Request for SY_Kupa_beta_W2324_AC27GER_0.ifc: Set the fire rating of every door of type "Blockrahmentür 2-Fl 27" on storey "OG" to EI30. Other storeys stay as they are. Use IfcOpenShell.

First a look at what the model holds.

```python
import ifcopenshell
import ifcopenshell.util.element

model = ifcopenshell.open("SY_Kupa_beta_W2324_AC27GER_0.ifc")
print(model.schema)
storey = next(s for s in model.by_type("IfcBuildingStorey") if s.Name == "OG")
doors = [e for e in ifcopenshell.util.element.get_decomposition(storey) if e.is_a("IfcDoor")]
seen = {}
for e in doors:
    element_type = ifcopenshell.util.element.get_type(e)
    key = (element_type.Name if element_type != e and element_type else None, ifcopenshell.util.element.get_pset(e, "Pset_DoorCommon", "FireRating"))
    seen[key] = seen.get(key, 0) + 1
for (name, value), count in sorted(seen.items(), key=str):
    print(count, "x", name, "|", value)
```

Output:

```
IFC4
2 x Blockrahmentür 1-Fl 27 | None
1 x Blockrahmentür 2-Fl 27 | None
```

```python
import ifcopenshell
import ifcopenshell.api.pset
import ifcopenshell.util.element

model = ifcopenshell.open("SY_Kupa_beta_W2324_AC27GER_0.ifc")

storey = next(s for s in model.by_type("IfcBuildingStorey") if s.Name == "OG")
doors = [e for e in ifcopenshell.util.element.get_decomposition(storey) if e.is_a("IfcDoor")]

count = 0
for e in doors:
    element_type = ifcopenshell.util.element.get_type(e)
    if element_type in (None, e) or element_type.Name != "Blockrahmentür 2-Fl 27":
        continue
    # add_pset returns the element's existing set when there is one.
    pset = ifcopenshell.api.pset.add_pset(model, product=e, name="Pset_DoorCommon")
    ifcopenshell.api.pset.edit_pset(model, pset=pset, properties={"FireRating": "EI30"})
    count += 1

print(count, "doors updated")

model.write("SY_Kupa_beta_W2324_AC27GER_0_rev.ifc")
```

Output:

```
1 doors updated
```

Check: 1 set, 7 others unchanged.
